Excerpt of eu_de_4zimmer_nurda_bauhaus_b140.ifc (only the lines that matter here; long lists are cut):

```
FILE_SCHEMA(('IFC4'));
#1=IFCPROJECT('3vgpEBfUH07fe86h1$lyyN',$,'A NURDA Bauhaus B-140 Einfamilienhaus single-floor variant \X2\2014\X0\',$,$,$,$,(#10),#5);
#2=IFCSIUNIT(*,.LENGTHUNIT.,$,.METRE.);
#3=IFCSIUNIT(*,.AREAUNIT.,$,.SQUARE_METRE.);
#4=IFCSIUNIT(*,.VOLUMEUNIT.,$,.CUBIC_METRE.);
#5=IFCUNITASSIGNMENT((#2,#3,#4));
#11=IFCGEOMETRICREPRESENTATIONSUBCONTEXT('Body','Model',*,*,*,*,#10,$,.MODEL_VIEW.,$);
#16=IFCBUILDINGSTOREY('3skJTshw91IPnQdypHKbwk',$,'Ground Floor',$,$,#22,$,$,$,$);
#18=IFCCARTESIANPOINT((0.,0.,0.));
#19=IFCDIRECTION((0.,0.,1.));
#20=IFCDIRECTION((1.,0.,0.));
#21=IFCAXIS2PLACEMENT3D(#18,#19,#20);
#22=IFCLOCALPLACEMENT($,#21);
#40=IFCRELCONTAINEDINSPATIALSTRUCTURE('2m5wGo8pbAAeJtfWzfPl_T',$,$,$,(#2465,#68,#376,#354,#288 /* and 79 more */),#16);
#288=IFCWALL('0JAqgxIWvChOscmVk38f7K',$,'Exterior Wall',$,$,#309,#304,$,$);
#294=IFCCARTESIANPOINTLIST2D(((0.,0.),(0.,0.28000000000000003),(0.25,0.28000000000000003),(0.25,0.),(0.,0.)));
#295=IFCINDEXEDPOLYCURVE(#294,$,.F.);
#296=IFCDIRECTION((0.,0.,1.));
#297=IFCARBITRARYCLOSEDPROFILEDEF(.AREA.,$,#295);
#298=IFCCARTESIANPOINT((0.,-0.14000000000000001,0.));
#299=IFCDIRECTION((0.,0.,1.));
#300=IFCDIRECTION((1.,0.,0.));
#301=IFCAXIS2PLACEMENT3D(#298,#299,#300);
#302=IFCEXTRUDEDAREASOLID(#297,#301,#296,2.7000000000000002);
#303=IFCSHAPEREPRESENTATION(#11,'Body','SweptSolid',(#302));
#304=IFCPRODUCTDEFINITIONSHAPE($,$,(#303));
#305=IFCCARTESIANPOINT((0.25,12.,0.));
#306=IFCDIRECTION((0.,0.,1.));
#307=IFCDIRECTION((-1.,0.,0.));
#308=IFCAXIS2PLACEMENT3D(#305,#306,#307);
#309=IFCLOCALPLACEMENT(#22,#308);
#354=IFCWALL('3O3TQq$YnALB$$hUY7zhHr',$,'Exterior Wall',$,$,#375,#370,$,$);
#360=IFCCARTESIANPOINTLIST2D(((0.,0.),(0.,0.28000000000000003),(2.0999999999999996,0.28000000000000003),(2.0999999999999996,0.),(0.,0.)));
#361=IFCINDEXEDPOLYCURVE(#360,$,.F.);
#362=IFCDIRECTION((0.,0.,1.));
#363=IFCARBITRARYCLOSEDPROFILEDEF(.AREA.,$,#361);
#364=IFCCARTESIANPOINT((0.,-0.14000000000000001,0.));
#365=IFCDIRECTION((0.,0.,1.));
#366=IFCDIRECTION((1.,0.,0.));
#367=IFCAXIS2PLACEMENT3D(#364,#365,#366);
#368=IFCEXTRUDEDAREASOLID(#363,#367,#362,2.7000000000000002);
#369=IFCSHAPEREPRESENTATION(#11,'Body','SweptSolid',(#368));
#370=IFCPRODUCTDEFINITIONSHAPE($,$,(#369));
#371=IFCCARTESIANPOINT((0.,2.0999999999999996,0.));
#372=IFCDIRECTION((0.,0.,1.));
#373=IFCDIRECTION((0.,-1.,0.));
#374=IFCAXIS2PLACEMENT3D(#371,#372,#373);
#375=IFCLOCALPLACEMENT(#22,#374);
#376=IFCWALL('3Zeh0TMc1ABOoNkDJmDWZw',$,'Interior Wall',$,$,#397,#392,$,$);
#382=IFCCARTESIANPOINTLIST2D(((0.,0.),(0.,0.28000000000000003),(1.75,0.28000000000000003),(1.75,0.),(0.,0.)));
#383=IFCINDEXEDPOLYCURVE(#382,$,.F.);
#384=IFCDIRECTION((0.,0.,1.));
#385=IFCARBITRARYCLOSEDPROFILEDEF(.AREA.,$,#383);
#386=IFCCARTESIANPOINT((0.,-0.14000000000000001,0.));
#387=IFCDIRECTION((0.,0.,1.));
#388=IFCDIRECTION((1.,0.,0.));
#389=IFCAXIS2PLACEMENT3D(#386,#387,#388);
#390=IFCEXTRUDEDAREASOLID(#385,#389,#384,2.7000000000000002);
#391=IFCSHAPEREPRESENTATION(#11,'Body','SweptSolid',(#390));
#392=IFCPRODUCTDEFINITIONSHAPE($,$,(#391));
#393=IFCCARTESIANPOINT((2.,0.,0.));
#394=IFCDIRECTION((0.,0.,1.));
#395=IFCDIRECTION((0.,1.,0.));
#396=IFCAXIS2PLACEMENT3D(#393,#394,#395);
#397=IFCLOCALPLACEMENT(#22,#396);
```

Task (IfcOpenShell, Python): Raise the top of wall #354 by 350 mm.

```python
import ifcopenshell
import ifcopenshell.geom
import ifcopenshell.util.representation
import ifcopenshell.util.shape

model = ifcopenshell.open("eu_de_4zimmer_nurda_bauhaus_b140.ifc")
settings = ifcopenshell.geom.settings()


def volume(element):
    """Net volume in cubic metres, openings subtracted."""
    shape = ifcopenshell.geom.create_shape(settings, element)
    return ifcopenshell.util.shape.get_volume(shape.geometry)


wall = model.by_id(354)
before = volume(wall)

body = ifcopenshell.util.representation.get_representation(wall, "Model", "Body")
solid = body.Items[0]
old_height = solid.Depth
solid.Depth += 0.35
after = volume(wall)

print(f"height {old_height:g} -> {solid.Depth:g}, volume {before:.3f} -> {after:.3f} m3")

model.write("eu_de_4zimmer_nurda_bauhaus_b140_edited.ifc")
```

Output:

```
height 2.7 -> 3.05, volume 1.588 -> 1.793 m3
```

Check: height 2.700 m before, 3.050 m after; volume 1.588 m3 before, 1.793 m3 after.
